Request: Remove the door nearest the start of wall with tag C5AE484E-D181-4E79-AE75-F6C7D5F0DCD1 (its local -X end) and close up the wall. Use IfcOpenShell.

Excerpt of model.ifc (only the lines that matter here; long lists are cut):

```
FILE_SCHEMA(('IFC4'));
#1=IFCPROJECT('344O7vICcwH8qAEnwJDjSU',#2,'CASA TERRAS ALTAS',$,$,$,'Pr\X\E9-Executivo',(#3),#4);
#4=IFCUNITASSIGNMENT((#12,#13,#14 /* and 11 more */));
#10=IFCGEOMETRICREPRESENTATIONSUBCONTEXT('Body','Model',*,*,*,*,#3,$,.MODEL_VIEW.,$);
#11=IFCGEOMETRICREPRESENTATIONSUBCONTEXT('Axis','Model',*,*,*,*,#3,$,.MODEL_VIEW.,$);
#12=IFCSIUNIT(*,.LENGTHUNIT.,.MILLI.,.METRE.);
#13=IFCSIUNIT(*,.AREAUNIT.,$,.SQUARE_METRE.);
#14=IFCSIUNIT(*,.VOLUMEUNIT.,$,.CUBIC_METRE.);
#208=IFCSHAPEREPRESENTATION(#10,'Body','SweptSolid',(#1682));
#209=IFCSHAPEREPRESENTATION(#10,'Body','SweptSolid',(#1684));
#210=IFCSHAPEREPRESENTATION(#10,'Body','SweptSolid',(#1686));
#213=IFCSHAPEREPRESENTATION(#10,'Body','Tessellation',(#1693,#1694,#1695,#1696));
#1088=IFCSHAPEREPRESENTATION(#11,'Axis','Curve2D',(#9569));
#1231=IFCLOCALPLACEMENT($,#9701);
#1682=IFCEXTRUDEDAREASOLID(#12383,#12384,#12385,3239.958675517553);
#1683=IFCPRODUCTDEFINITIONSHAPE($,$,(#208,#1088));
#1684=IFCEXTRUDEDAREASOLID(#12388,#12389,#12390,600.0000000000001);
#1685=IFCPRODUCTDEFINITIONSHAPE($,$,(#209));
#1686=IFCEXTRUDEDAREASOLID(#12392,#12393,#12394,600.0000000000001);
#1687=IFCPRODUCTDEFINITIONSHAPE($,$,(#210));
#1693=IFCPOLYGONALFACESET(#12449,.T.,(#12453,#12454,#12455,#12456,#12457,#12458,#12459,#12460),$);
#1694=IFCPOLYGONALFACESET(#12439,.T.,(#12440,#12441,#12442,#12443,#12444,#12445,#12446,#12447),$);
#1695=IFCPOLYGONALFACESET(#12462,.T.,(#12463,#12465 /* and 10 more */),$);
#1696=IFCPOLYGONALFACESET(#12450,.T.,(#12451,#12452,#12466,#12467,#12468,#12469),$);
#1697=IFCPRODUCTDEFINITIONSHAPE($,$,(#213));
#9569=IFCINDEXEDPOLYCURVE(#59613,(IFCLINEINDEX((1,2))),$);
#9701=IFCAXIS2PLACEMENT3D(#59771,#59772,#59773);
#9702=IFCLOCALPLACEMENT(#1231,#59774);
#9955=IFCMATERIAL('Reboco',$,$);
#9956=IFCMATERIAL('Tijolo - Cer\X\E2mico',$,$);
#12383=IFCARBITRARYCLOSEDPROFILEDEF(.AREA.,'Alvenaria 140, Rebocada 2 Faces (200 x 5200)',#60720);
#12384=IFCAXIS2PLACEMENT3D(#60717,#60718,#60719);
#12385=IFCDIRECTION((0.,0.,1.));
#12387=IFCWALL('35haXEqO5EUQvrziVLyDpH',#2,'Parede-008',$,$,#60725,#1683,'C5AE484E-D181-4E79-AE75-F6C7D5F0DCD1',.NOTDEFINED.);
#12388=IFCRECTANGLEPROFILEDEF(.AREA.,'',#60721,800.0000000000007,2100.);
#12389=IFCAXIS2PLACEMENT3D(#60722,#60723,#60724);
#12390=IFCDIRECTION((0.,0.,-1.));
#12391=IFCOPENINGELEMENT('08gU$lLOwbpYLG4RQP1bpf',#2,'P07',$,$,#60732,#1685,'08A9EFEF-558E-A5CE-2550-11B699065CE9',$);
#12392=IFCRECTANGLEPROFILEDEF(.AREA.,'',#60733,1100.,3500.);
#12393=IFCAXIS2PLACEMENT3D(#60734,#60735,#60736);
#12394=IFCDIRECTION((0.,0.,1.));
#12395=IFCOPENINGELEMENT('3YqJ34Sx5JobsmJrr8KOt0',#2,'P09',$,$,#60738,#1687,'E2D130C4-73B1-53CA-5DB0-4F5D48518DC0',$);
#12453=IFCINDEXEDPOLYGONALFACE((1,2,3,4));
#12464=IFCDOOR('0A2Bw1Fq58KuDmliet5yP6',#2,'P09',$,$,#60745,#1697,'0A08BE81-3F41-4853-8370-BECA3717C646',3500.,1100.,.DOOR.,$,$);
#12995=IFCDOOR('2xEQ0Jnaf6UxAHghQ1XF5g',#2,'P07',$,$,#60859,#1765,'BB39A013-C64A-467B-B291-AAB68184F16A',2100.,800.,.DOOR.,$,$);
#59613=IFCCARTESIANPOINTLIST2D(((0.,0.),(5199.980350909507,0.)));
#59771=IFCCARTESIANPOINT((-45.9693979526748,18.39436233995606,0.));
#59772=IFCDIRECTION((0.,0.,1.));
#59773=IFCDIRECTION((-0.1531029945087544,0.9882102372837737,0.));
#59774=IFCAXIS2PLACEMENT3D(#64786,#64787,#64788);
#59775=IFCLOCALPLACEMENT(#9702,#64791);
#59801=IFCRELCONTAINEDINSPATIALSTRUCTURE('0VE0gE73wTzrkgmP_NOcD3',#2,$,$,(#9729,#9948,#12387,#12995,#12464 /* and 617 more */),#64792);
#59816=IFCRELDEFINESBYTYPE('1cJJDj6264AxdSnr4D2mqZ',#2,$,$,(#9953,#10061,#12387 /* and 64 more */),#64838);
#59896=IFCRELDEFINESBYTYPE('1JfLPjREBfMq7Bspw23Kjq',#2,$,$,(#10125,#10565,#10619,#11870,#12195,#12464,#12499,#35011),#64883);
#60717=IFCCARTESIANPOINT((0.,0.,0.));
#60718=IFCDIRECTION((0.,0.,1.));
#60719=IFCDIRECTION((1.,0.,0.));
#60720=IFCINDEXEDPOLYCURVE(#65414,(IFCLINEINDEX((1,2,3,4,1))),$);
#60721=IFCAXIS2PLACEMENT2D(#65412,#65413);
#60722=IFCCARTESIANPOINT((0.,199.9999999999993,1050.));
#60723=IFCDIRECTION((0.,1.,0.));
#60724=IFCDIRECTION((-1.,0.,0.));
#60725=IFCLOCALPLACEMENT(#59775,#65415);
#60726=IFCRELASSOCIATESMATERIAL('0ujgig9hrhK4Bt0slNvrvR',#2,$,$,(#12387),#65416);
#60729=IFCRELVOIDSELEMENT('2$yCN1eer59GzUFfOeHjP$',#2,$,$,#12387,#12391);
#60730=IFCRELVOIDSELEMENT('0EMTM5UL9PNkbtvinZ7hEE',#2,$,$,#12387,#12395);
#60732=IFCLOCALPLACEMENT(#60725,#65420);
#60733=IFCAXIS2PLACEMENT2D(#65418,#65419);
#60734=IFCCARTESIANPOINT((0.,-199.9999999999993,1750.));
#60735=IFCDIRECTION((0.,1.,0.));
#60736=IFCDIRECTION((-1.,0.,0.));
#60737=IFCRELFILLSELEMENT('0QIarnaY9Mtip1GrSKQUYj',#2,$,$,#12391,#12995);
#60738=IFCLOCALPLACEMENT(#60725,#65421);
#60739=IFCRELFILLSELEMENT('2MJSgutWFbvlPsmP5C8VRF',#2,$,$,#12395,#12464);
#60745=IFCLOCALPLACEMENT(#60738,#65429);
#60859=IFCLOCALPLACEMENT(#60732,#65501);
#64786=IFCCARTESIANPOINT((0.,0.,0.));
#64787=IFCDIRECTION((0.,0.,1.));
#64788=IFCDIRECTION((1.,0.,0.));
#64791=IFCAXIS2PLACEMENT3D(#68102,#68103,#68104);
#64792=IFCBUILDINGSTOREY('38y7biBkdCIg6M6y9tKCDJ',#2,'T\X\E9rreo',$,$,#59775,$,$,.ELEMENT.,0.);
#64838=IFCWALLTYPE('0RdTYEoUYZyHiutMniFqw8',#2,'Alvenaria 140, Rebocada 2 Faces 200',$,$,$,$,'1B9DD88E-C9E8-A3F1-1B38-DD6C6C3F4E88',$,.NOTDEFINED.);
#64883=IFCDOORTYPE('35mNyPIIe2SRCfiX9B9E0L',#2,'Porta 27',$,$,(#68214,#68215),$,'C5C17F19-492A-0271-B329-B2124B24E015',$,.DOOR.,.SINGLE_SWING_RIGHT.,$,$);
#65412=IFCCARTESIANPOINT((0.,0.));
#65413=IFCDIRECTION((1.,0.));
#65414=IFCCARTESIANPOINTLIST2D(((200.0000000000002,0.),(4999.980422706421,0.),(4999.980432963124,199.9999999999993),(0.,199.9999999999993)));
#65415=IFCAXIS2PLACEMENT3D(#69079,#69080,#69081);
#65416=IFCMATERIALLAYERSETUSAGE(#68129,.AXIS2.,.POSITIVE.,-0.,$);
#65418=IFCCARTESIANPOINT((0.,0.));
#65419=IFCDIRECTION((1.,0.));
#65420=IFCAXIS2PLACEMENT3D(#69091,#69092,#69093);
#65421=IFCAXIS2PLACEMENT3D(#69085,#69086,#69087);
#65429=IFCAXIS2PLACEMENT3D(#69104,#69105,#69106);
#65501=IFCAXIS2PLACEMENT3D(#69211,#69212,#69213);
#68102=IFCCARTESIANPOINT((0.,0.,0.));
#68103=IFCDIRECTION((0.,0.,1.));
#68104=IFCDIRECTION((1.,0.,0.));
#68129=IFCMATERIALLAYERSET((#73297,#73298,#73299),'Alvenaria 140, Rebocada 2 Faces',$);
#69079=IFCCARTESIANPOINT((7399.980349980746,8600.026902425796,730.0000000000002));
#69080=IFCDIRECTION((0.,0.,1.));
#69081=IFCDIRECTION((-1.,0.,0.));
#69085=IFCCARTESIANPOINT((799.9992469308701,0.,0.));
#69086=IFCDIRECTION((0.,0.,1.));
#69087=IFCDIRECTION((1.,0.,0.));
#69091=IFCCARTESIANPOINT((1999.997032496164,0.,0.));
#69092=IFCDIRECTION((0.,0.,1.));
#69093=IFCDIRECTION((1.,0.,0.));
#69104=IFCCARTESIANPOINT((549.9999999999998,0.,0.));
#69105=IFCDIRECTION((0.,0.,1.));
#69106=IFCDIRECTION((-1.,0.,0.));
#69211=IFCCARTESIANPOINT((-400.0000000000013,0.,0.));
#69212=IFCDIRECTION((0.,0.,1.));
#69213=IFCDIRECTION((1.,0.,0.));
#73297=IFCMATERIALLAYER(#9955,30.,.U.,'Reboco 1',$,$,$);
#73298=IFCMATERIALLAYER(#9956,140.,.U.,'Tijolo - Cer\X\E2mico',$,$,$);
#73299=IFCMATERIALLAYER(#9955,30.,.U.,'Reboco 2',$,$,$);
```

```python
import ifcopenshell
import ifcopenshell.api.feature
import ifcopenshell.api.root
import ifcopenshell.geom
import ifcopenshell.util.shape

model = ifcopenshell.open("model.ifc")
settings = ifcopenshell.geom.settings()


def volume(element):
    """Net volume in cubic metres, openings subtracted."""
    shape = ifcopenshell.geom.create_shape(settings, element)
    return ifcopenshell.util.shape.get_volume(shape.geometry)


door = model.by_id(12464)
opening = door.FillsVoids[0].RelatingOpeningElement
wall = opening.VoidsElements[0].RelatingBuildingElement
before = volume(wall)

ifcopenshell.api.root.remove_product(model, product=door)
ifcopenshell.api.feature.remove_feature(model, feature=opening)

after = volume(wall)

print(f"wall volume {before:.3f} -> {after:.3f} m3")

model.write("model-out.ifc")
```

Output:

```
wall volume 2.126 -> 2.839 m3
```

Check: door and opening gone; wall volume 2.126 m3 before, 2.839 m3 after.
